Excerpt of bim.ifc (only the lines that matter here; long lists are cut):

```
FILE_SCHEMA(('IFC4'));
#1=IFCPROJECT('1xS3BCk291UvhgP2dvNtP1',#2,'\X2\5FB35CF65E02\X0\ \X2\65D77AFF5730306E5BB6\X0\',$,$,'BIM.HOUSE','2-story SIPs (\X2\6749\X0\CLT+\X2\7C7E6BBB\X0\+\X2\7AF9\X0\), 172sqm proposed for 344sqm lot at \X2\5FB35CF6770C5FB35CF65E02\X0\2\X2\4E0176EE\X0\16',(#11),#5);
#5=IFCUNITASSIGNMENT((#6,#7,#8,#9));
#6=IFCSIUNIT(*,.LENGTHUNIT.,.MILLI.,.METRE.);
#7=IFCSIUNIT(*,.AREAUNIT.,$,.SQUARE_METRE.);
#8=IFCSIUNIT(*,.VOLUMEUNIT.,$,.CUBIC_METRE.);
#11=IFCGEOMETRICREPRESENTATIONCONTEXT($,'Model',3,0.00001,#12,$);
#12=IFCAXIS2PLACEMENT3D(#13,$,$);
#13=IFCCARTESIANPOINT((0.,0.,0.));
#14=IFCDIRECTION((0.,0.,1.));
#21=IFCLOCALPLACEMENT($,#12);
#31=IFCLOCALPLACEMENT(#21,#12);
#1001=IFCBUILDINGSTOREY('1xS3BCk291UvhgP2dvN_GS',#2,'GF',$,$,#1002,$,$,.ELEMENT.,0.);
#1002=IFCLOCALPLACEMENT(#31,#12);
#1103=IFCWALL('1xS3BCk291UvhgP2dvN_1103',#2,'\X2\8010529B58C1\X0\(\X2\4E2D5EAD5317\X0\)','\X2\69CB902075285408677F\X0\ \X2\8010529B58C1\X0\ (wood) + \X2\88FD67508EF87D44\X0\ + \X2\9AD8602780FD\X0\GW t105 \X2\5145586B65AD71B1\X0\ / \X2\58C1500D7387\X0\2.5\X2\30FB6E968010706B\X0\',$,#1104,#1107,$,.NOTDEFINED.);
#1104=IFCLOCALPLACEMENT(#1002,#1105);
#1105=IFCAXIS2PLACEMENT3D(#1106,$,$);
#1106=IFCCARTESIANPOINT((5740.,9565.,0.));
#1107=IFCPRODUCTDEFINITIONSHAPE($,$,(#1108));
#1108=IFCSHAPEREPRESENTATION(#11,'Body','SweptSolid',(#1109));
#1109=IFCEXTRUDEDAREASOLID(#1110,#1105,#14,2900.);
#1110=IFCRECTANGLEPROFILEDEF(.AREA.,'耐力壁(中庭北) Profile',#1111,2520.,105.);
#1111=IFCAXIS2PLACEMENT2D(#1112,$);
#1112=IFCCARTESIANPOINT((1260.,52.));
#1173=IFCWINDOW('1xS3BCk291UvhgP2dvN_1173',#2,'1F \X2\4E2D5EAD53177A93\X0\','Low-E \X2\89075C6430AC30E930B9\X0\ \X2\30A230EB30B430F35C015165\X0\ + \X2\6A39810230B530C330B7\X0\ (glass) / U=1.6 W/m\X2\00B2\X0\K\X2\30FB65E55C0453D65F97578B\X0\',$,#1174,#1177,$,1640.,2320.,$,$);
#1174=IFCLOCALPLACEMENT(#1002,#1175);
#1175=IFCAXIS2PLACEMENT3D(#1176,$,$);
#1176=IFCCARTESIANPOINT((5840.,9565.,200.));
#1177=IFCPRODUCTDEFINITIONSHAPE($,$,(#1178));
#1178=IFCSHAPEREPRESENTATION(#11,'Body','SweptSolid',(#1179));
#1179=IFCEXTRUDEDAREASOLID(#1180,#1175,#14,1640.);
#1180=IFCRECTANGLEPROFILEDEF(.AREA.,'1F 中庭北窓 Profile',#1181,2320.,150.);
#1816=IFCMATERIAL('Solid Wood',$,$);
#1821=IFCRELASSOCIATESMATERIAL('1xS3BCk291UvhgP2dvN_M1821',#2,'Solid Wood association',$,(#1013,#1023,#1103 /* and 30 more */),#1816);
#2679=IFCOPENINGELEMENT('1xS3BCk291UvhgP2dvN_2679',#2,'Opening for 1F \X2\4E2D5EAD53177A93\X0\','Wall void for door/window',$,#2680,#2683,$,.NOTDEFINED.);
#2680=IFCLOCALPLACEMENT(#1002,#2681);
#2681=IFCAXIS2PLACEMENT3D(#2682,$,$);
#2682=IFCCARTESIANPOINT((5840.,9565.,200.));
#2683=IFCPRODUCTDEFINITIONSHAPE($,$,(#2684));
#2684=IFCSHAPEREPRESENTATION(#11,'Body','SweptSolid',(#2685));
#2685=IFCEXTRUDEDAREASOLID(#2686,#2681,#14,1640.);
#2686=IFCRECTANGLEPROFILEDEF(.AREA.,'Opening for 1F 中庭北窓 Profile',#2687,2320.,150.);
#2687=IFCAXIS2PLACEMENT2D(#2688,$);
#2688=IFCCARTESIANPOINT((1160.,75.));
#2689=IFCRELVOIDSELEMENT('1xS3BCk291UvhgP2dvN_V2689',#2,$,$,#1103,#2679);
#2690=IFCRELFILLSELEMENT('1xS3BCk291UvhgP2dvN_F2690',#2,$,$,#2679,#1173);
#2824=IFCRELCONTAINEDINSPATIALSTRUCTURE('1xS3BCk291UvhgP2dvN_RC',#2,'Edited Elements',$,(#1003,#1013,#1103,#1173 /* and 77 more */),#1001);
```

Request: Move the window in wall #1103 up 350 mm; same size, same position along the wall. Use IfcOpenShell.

```python
import numpy as np
import ifcopenshell
import ifcopenshell.api.geometry
import ifcopenshell.util.placement
import ifcopenshell.util.unit

model = ifcopenshell.open("bim.ifc")
unit_scale = ifcopenshell.util.unit.calculate_unit_scale(model)

window = model.by_guid("1xS3BCk291UvhgP2dvN_1173")
opening = window.FillsVoids[0].RelatingOpeningElement
dz = 350.0

shift = np.array([0.0, 0.0, dz])
# The window is not placed relative to its opening, so move both.
for product in (opening, window):
    matrix = ifcopenshell.util.placement.get_local_placement(product.ObjectPlacement)
    matrix[:3, 3] += shift
    ifcopenshell.api.geometry.edit_object_placement(model, product=product, matrix=matrix, is_si=False)

print(f"moved by {dz * unit_scale:+.3f} m")

model.write("bim_rev.ifc")
```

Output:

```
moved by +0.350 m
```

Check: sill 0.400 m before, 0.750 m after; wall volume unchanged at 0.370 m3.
